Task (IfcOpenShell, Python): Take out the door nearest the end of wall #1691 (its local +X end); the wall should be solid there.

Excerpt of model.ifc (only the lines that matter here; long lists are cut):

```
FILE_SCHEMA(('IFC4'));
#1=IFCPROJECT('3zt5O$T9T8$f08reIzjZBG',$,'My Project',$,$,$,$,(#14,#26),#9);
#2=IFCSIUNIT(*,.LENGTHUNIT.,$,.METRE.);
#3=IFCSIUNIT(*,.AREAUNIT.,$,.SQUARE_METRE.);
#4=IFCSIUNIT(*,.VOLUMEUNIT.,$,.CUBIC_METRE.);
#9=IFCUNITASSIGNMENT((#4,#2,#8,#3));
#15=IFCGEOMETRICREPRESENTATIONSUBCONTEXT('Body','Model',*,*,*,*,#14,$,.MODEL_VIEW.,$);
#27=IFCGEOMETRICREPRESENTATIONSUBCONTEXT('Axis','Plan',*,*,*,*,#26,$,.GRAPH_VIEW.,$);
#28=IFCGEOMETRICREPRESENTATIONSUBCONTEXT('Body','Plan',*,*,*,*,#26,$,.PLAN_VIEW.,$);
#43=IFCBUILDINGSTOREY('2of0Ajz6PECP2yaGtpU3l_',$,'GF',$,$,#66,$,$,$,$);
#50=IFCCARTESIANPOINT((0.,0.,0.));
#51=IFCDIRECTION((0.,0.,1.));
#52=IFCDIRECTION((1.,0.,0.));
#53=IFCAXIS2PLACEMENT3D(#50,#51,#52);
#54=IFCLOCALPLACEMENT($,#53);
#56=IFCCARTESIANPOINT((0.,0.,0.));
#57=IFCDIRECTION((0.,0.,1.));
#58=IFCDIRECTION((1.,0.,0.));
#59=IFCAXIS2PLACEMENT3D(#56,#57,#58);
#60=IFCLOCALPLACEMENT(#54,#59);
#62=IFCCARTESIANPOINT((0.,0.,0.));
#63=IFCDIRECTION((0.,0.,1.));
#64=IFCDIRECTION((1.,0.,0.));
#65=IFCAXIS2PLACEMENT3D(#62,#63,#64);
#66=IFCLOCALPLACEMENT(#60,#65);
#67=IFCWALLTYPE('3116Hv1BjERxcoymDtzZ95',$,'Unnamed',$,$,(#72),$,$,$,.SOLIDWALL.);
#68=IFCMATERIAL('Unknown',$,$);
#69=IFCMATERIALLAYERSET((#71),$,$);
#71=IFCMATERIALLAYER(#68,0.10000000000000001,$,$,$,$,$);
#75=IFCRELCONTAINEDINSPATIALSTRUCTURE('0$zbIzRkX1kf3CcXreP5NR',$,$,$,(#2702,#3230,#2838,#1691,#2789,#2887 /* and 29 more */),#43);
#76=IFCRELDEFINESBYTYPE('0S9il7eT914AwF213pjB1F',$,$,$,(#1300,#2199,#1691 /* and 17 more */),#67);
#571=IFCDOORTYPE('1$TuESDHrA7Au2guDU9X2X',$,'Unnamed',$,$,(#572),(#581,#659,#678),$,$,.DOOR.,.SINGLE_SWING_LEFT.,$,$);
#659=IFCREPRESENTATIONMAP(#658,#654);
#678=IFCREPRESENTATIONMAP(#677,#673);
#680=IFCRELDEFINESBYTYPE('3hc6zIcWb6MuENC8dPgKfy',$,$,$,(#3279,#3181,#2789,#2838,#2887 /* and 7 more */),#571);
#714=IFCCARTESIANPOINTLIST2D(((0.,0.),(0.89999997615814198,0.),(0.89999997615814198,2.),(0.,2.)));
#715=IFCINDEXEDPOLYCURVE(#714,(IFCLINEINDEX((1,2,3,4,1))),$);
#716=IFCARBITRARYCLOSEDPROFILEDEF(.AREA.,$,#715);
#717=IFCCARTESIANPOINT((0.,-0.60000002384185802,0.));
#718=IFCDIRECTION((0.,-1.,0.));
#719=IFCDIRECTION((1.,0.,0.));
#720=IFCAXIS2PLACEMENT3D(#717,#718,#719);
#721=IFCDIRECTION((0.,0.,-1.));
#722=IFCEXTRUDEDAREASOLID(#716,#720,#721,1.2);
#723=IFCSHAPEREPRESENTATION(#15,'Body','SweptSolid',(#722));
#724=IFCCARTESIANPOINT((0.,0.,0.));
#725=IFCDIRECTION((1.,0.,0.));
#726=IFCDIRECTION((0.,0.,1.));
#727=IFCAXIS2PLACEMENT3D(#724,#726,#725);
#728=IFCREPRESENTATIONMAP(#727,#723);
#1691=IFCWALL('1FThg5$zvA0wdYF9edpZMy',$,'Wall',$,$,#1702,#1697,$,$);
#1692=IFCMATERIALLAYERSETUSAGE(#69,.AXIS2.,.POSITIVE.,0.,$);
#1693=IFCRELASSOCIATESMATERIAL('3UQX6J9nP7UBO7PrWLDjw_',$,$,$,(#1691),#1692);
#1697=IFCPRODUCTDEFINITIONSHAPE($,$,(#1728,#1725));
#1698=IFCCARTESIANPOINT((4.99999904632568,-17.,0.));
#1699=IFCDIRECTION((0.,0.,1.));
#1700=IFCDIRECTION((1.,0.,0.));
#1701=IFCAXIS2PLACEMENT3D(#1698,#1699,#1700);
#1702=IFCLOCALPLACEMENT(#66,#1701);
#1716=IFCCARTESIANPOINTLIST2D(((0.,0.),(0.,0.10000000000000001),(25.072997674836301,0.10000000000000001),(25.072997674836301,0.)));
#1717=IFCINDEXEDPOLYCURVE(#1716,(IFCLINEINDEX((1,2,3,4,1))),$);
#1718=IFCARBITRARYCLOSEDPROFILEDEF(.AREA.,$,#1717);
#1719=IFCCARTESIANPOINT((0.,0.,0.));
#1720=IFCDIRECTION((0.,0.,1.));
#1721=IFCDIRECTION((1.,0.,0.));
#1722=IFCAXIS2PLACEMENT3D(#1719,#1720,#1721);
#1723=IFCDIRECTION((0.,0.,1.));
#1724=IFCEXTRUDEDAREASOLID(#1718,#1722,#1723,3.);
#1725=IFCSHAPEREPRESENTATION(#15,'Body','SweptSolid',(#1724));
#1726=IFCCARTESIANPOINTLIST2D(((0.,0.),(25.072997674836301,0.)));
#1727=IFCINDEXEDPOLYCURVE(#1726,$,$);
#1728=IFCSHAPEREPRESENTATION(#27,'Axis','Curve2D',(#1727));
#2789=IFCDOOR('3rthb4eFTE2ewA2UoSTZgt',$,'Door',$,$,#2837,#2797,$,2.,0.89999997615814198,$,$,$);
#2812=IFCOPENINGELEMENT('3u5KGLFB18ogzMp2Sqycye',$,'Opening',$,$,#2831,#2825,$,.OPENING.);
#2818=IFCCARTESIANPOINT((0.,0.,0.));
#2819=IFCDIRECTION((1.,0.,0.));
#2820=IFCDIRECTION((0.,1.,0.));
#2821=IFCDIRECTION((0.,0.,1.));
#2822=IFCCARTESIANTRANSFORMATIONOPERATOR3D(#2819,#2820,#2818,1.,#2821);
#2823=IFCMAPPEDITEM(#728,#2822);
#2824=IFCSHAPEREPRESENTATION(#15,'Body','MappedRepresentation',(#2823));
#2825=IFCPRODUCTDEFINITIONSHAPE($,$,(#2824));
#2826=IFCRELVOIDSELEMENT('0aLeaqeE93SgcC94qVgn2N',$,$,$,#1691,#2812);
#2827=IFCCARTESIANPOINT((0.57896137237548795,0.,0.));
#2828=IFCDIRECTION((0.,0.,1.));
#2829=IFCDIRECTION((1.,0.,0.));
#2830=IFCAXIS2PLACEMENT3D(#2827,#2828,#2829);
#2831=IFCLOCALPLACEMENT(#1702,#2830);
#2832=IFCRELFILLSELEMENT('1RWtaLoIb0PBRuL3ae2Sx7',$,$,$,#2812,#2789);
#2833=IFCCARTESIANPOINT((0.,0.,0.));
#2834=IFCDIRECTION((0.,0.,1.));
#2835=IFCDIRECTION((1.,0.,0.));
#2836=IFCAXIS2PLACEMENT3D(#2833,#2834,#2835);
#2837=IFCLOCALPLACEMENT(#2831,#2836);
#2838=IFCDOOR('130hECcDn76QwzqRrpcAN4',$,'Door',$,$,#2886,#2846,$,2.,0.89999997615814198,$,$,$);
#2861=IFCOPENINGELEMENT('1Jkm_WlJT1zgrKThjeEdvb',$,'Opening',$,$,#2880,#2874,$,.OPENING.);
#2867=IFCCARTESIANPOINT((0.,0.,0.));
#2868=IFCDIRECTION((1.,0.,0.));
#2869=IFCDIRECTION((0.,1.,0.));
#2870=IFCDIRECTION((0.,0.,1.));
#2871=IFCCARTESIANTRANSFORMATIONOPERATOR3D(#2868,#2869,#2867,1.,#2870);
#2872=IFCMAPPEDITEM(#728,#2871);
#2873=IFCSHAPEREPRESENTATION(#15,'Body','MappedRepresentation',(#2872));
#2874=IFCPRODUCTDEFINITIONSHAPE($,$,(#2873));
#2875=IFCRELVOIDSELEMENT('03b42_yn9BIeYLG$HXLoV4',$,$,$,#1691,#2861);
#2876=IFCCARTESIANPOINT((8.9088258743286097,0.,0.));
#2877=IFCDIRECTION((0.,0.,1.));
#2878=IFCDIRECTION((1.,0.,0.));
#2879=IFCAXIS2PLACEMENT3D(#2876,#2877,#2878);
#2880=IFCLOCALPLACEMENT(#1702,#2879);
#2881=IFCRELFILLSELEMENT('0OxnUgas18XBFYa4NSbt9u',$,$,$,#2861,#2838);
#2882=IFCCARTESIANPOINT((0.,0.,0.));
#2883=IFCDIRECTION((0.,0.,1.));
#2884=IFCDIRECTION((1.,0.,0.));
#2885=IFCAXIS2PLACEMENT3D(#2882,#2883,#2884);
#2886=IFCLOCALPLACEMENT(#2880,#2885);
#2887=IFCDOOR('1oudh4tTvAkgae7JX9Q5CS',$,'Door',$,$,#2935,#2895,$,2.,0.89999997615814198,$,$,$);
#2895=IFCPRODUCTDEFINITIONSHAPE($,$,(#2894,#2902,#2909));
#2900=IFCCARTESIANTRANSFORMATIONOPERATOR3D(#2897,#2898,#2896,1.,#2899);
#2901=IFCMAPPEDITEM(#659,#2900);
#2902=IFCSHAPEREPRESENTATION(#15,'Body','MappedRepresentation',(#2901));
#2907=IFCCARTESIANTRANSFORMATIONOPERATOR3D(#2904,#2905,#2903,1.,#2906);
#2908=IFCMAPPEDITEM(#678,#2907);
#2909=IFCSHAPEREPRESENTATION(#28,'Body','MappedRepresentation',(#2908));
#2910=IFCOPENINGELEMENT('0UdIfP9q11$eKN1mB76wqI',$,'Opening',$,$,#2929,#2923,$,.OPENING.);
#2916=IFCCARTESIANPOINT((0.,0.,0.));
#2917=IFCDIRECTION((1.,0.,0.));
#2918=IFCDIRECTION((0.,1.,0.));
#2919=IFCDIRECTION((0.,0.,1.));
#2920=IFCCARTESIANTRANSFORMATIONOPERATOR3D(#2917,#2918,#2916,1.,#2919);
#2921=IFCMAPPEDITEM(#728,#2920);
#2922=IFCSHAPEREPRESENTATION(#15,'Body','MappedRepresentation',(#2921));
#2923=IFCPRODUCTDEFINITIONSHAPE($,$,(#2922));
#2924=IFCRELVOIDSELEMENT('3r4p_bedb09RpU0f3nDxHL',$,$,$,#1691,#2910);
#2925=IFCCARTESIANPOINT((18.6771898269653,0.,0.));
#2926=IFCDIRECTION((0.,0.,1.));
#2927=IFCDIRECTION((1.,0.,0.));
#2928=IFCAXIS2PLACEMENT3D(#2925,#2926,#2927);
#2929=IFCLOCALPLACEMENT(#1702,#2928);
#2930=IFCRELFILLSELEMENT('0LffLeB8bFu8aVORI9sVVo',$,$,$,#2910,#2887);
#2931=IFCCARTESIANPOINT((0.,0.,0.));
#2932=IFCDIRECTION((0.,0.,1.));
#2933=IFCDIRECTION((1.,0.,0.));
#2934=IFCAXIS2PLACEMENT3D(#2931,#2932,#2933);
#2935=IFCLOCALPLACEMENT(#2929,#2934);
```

```python
import ifcopenshell
import ifcopenshell.api.feature
import ifcopenshell.api.root
import ifcopenshell.geom
import ifcopenshell.util.shape

model = ifcopenshell.open("model.ifc")
settings = ifcopenshell.geom.settings()


def volume(element):
    """Net volume in cubic metres, openings subtracted."""
    shape = ifcopenshell.geom.create_shape(settings, element)
    return ifcopenshell.util.shape.get_volume(shape.geometry)


door = model.by_id(2887)
opening = door.FillsVoids[0].RelatingOpeningElement
wall = opening.VoidsElements[0].RelatingBuildingElement
before = volume(wall)

ifcopenshell.api.root.remove_product(model, product=door)
ifcopenshell.api.feature.remove_feature(model, feature=opening)

after = volume(wall)

print(f"wall volume {before:.3f} -> {after:.3f} m3")

model.write("model_edited.ifc")
```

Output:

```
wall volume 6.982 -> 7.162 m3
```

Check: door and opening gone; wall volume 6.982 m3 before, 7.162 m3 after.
